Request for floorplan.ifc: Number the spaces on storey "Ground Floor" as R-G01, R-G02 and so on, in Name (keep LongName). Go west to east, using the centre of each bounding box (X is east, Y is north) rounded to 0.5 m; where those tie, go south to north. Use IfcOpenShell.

First a look at what the model holds.

```python
import ifcopenshell
import ifcopenshell.util.element
import ifcopenshell.util.placement

model = ifcopenshell.open("floorplan.ifc")
print(model.schema)
storey = next(s for s in model.by_type("IfcBuildingStorey") if s.Name == "Ground Floor")
spaces = [e for e in ifcopenshell.util.element.get_decomposition(storey) if e.is_a("IfcSpace")]
for e in sorted(spaces, key=lambda e: e.id()):
    origin = ifcopenshell.util.placement.get_local_placement(e.ObjectPlacement)[:3, 3]
    print(e.id(), e.Name, e.LongName, origin.round(2) + 0.0, sep=" | ")
```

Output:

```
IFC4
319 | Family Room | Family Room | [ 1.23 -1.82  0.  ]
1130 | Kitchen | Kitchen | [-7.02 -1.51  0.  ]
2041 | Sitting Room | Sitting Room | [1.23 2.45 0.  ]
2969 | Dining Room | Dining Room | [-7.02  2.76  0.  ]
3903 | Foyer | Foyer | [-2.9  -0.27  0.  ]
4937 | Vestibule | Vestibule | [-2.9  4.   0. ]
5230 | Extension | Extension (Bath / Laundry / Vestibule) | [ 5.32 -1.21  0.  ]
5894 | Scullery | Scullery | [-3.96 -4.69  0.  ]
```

```python
import ifcopenshell
import ifcopenshell.geom
import ifcopenshell.util.element
import ifcopenshell.util.shape

model = ifcopenshell.open("floorplan.ifc")
settings = ifcopenshell.geom.settings()
settings.set("use-world-coords", True)


def centre(element):
    shape = ifcopenshell.geom.create_shape(settings, element)
    return ifcopenshell.util.shape.get_bbox_centroid(shape.geometry)


storey = next(s for s in model.by_type("IfcBuildingStorey") if s.Name == "Ground Floor")
spaces = [e for e in ifcopenshell.util.element.get_decomposition(storey) if e.is_a("IfcSpace")]

# Insertion points can sit at a corner or the storey origin, so sort by the geometry (in metres).
centres = {e: centre(e) for e in spaces}
spaces.sort(key=lambda e: (round(centres[e][0] / 0.5), centres[e][1]))

for i, e in enumerate(spaces, start=1):
    number = f"R-G{i:02d}"
    e.Name = number
    print(e.id(), number)

model.write("floorplan-out.ifc")
```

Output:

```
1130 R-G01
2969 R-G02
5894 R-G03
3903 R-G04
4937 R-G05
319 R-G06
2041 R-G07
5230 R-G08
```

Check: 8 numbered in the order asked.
